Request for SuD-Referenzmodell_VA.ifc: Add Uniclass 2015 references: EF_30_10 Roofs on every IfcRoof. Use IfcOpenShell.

First a look at what the model holds.

```python
import ifcopenshell

model = ifcopenshell.open("SuD-Referenzmodell_VA.ifc")
print(model.schema)
print("classifications:", [c.Name for c in model.by_type("IfcClassification")])
for ifc_class in ("IfcDoor", "IfcRoof", "IfcStair", "IfcWall", "IfcWindow"):
    print(ifc_class, len(model.by_type(ifc_class)))
```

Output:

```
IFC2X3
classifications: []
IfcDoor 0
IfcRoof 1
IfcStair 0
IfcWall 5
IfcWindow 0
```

```python
import ifcopenshell
import ifcopenshell.api.classification

model = ifcopenshell.open("SuD-Referenzmodell_VA.ifc")

# IFC2X3 requires Source and Edition and has no link from the project to the system.
system = model.create_entity("IfcClassification", Source="NBS", Edition="2015", Name="Uniclass 2015")

codes = {
    "IfcRoof": ("EF_30_10", "Roofs"),
}
for ifc_class, (code, name) in codes.items():
    products = model.by_type(ifc_class)
    ifcopenshell.api.classification.add_reference(
        model, products=products, classification=system, identification=code, name=name
    )
    print(code, len(products))

model.write("SuD-Referenzmodell_VA_v2.ifc")
```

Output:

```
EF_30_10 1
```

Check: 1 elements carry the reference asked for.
